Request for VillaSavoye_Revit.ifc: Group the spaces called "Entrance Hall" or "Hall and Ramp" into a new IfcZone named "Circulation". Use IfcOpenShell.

First a look at what the model holds.

```python
import ifcopenshell

model = ifcopenshell.open("VillaSavoye_Revit.ifc")
print(model.schema)
seen = {}
for space in model.by_type("IfcSpace"):
    seen[space.LongName] = seen.get(space.LongName, 0) + 1
for name, count in sorted(seen.items(), key=str):
    print(count, "x", name)
print("zones:", [z.Name for z in model.by_type("IfcZone")][:20])
```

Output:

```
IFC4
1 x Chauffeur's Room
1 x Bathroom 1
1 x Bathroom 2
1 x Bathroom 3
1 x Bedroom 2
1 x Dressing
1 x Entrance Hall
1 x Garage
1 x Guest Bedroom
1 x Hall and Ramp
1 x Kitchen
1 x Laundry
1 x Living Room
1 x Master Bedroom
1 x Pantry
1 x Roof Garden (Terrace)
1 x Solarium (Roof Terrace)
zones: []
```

```python
import ifcopenshell
import ifcopenshell.api.group
import ifcopenshell.api.root

model = ifcopenshell.open("VillaSavoye_Revit.ifc")

names = {"Entrance Hall", "Hall and Ramp"}
spaces = [s for s in model.by_type("IfcSpace") if s.LongName in names]

zone = ifcopenshell.api.root.create_entity(model, ifc_class="IfcZone", name="Circulation")
ifcopenshell.api.group.assign_group(model, products=spaces, group=zone)
print(len(spaces), "spaces in", zone.Name)

model.write("VillaSavoye_Revit_rev.ifc")
```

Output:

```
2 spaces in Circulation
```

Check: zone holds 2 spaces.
